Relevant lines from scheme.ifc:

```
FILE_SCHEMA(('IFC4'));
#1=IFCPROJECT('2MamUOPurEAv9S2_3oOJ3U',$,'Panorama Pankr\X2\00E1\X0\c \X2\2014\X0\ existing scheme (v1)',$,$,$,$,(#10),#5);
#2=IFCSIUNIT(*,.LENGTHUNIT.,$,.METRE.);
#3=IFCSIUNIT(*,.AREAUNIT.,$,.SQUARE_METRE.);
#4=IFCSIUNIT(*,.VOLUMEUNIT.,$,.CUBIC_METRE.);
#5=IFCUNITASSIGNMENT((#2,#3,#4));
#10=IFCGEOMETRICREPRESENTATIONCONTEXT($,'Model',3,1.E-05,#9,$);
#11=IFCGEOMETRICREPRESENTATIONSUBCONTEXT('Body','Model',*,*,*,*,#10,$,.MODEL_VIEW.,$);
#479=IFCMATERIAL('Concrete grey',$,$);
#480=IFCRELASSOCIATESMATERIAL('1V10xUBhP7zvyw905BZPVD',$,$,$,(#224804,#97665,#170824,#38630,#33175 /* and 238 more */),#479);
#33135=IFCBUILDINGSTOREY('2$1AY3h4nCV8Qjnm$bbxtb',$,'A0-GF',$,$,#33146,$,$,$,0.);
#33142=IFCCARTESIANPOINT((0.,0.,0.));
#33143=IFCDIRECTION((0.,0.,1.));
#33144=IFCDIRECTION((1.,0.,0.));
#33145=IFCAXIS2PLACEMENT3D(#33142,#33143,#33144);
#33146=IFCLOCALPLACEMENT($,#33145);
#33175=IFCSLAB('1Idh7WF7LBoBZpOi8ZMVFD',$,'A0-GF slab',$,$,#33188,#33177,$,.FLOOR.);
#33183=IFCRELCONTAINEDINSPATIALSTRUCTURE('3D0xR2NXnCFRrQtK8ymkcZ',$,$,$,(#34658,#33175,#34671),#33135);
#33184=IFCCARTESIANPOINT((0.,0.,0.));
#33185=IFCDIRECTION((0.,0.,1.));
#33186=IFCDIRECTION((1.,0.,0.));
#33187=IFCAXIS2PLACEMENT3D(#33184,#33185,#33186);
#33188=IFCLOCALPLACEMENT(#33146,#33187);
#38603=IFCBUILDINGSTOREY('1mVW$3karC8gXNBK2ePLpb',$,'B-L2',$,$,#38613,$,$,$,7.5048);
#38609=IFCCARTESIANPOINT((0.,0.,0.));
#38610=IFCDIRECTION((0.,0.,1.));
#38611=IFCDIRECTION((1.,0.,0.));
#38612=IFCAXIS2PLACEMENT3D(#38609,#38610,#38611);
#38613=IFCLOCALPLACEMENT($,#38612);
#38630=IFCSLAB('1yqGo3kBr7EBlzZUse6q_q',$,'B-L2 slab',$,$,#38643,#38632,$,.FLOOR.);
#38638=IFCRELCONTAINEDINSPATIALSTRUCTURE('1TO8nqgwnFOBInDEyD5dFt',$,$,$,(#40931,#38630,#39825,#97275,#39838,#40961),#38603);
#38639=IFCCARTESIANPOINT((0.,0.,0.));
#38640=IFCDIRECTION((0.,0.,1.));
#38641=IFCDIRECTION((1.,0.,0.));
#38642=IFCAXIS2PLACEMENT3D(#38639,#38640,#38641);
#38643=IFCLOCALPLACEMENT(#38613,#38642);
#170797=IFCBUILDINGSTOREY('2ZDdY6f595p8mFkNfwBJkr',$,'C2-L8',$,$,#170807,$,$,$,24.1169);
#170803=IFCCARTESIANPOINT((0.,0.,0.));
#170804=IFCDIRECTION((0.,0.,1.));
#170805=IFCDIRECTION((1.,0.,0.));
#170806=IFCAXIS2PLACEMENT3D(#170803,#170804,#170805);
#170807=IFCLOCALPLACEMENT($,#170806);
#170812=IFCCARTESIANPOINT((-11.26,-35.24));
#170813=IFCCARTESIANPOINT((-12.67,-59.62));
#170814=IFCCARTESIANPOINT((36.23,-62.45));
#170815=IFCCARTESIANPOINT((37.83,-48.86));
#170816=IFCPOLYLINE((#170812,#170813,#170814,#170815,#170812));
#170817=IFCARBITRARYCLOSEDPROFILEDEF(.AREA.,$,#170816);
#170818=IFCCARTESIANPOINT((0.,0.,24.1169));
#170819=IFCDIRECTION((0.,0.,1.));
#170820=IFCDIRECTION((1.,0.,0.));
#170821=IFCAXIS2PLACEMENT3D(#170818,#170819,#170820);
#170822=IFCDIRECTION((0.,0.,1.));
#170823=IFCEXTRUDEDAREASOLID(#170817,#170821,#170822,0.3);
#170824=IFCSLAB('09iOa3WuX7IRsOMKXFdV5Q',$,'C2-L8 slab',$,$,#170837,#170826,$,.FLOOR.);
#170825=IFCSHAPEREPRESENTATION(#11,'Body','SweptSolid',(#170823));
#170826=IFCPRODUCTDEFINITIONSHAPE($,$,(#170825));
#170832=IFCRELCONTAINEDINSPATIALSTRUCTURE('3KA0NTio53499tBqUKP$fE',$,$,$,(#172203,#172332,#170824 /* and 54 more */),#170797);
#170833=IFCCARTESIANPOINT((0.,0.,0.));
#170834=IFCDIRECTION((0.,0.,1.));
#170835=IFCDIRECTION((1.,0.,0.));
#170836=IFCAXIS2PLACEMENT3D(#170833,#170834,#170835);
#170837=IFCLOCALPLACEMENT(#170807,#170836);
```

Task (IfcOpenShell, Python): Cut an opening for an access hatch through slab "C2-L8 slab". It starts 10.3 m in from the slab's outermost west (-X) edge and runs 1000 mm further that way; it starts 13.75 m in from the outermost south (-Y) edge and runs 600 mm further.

```python
import numpy as np
import ifcopenshell
import ifcopenshell.api.feature
import ifcopenshell.api.geometry
import ifcopenshell.api.root
import ifcopenshell.geom
import ifcopenshell.util.placement
import ifcopenshell.util.representation
import ifcopenshell.util.shape
import ifcopenshell.util.unit

model = ifcopenshell.open("scheme.ifc")
unit_scale = ifcopenshell.util.unit.calculate_unit_scale(model)
settings = ifcopenshell.geom.settings()


def volume(element):
    """Net volume in cubic metres, openings subtracted."""
    shape = ifcopenshell.geom.create_shape(settings, element)
    return ifcopenshell.util.shape.get_volume(shape.geometry)


slab = model.by_guid("09iOa3WuX7IRsOMKXFdV5Q")
before = volume(slab)

# Extent in the slab's own axes, in metres. The edges named are its -X and -Y sides.
slab_shape = ifcopenshell.geom.create_shape(settings, slab)
vertices = ifcopenshell.util.shape.get_vertices(slab_shape.geometry)
x_min, y_min, bottom = vertices.min(axis=0)
top = vertices[:, 2].max()

opening = ifcopenshell.api.root.create_entity(model, ifc_class="IfcOpeningElement", name="Access hatch opening", predefined_type="OPENING")
context = ifcopenshell.util.representation.get_context(model, "Model", "Body", "MODEL_VIEW")
width, depth = 1, 0.6
outline = [(0.0, 0.0), (width, 0.0), (width, depth), (0.0, depth), (0.0, 0.0)]
# Overshoot both faces by 50 mm so the cut is clean.
shape = ifcopenshell.api.geometry.add_slab_representation(
    model, context=context, depth=top - bottom + 0.1, polyline=outline
)
ifcopenshell.api.geometry.assign_representation(model, product=opening, representation=shape)

matrix = ifcopenshell.util.placement.get_local_placement(slab.ObjectPlacement)
matrix[:, 3] = matrix @ np.append(np.array([x_min + 10.3, y_min + 13.75, bottom - 0.05]) / unit_scale, 1.0)
ifcopenshell.api.geometry.edit_object_placement(model, product=opening, matrix=matrix, is_si=False)
ifcopenshell.api.feature.add_feature(model, feature=opening, element=slab)

after = volume(slab)

print(f"slab volume {before:.3f} -> {after:.3f} m3")

model.write("scheme-out.ifc")
```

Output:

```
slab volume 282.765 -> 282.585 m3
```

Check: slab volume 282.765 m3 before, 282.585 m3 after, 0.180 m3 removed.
